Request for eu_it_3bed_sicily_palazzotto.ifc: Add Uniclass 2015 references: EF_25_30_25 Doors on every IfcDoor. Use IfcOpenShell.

First a look at what the model holds.

```python
import ifcopenshell

model = ifcopenshell.open("eu_it_3bed_sicily_palazzotto.ifc")
print(model.schema)
print("classifications:", [c.Name for c in model.by_type("IfcClassification")])
for ifc_class in ("IfcDoor", "IfcRoof", "IfcStair", "IfcWall", "IfcWindow"):
    print(ifc_class, len(model.by_type(ifc_class)))
```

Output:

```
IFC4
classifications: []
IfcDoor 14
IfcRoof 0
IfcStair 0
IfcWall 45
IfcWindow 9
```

```python
import ifcopenshell
import ifcopenshell.api.classification

model = ifcopenshell.open("eu_it_3bed_sicily_palazzotto.ifc")

system = ifcopenshell.api.classification.add_classification(model, classification="Uniclass 2015")

codes = {
    "IfcDoor": ("EF_25_30_25", "Doors"),
}
for ifc_class, (code, name) in codes.items():
    products = model.by_type(ifc_class)
    ifcopenshell.api.classification.add_reference(
        model, products=products, classification=system, identification=code, name=name
    )
    print(code, len(products))

model.write("eu_it_3bed_sicily_palazzotto-out.ifc")
```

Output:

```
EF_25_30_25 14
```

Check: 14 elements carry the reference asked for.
